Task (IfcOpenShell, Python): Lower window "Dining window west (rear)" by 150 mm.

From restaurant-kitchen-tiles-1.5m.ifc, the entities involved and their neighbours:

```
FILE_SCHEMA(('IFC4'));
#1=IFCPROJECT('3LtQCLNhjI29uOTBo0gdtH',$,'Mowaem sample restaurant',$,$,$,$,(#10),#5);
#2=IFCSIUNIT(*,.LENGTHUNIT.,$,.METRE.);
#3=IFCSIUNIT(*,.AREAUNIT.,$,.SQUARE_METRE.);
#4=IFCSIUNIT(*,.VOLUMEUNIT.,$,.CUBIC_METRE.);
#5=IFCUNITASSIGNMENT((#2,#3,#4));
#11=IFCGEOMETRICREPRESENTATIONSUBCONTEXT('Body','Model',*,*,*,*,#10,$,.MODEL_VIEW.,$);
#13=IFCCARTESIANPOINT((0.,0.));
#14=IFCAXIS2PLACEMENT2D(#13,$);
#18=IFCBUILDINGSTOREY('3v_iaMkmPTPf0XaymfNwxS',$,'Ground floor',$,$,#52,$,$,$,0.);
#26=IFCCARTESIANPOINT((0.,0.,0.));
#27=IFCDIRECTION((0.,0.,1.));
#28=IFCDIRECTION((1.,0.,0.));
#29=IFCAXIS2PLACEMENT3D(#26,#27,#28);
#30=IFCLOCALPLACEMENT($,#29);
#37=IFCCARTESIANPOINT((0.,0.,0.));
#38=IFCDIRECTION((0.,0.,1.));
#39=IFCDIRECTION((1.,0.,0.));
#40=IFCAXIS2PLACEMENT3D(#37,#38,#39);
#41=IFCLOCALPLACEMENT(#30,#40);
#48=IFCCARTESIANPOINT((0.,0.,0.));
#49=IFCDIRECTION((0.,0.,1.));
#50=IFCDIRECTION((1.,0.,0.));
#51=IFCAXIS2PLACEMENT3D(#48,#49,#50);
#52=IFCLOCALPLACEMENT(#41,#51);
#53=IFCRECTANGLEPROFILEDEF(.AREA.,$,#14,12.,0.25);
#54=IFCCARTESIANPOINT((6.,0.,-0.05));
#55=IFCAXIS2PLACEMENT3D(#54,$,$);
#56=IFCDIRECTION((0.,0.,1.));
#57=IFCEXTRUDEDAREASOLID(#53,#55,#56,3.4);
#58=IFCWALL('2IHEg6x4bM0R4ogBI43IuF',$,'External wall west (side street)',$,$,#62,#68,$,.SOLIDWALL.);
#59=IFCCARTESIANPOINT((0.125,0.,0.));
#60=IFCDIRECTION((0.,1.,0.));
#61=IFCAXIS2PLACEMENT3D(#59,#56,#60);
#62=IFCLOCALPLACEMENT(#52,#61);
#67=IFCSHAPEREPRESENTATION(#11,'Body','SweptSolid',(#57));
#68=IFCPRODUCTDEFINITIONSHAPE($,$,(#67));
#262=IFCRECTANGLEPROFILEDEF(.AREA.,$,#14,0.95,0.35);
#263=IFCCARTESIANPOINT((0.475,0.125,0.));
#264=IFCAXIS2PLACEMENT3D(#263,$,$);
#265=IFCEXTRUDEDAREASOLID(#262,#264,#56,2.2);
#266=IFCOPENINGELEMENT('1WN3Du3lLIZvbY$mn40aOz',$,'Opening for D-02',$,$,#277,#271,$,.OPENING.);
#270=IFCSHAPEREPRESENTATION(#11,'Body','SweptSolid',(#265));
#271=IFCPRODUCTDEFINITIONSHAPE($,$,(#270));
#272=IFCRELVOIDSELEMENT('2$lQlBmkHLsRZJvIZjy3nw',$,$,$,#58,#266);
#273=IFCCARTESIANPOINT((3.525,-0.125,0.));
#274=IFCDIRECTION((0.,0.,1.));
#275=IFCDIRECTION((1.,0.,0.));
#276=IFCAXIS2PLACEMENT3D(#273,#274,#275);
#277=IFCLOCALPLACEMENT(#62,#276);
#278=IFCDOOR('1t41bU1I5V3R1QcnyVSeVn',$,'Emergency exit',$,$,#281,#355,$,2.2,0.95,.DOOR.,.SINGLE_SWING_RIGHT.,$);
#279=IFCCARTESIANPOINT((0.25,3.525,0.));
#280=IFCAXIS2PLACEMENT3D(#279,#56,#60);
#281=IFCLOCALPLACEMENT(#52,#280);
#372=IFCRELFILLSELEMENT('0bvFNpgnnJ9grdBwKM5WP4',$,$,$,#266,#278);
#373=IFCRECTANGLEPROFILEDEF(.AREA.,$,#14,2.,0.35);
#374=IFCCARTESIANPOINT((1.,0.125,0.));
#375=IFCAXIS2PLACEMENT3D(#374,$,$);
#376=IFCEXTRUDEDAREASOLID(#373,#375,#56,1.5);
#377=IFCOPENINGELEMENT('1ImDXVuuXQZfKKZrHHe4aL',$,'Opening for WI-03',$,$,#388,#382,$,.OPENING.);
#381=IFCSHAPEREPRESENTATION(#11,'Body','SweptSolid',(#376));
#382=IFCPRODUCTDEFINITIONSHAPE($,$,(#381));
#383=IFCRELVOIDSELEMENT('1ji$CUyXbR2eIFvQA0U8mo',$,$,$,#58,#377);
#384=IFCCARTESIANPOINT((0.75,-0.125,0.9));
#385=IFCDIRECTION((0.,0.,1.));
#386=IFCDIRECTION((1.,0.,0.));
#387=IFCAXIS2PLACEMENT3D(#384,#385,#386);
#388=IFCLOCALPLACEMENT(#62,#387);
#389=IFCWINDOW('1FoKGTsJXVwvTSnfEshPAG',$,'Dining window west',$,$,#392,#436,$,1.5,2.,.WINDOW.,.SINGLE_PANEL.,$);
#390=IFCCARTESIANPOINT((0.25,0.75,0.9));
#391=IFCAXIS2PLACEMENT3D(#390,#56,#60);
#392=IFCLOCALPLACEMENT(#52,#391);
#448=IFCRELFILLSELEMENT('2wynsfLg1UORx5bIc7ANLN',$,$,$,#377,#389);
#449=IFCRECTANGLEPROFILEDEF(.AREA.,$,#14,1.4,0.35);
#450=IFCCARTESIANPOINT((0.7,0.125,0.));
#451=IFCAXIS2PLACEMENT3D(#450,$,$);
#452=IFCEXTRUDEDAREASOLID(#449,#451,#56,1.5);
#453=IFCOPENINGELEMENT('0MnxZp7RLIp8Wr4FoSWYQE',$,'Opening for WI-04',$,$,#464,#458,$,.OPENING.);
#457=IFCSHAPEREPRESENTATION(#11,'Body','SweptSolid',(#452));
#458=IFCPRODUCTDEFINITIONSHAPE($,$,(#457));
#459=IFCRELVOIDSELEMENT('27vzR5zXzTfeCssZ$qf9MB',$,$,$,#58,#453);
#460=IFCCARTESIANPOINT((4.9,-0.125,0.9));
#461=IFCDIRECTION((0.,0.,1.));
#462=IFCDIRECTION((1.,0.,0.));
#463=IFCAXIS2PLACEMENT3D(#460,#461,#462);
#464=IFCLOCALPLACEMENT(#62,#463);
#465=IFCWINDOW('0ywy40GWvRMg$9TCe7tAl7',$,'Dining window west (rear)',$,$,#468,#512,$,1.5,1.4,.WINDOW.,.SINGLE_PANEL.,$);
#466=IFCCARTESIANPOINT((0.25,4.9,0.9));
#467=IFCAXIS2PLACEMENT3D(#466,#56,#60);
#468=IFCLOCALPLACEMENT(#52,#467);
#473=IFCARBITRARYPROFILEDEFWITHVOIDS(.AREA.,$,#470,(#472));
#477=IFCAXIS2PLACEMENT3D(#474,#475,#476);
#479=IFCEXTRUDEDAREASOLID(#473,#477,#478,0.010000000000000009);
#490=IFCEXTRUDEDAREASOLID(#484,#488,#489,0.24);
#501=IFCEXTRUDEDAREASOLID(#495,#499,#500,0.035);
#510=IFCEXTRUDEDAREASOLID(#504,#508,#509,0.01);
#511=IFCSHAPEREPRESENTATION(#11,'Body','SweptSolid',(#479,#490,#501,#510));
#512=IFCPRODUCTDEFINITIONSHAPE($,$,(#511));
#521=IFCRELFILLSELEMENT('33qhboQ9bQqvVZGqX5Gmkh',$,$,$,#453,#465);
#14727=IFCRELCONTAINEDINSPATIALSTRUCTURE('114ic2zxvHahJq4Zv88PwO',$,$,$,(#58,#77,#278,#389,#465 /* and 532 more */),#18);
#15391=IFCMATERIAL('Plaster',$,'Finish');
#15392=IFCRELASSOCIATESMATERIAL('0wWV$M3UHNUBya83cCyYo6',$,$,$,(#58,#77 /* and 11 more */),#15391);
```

```python
import numpy as np
import ifcopenshell
import ifcopenshell.api.geometry
import ifcopenshell.util.placement
import ifcopenshell.util.unit

model = ifcopenshell.open("restaurant-kitchen-tiles-1.5m.ifc")
unit_scale = ifcopenshell.util.unit.calculate_unit_scale(model)

window = model.by_id(465)
opening = window.FillsVoids[0].RelatingOpeningElement
dz = -0.15 / unit_scale

shift = np.array([0.0, 0.0, dz])
# The window is not placed relative to its opening, so move both.
for product in (opening, window):
    matrix = ifcopenshell.util.placement.get_local_placement(product.ObjectPlacement)
    matrix[:3, 3] += shift
    ifcopenshell.api.geometry.edit_object_placement(model, product=product, matrix=matrix, is_si=False)

print(f"moved by {dz * unit_scale:+.3f} m")

model.write("restaurant-kitchen-tiles-1.5m-out.ifc")
```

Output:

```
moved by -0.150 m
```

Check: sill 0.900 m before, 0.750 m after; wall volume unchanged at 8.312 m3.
